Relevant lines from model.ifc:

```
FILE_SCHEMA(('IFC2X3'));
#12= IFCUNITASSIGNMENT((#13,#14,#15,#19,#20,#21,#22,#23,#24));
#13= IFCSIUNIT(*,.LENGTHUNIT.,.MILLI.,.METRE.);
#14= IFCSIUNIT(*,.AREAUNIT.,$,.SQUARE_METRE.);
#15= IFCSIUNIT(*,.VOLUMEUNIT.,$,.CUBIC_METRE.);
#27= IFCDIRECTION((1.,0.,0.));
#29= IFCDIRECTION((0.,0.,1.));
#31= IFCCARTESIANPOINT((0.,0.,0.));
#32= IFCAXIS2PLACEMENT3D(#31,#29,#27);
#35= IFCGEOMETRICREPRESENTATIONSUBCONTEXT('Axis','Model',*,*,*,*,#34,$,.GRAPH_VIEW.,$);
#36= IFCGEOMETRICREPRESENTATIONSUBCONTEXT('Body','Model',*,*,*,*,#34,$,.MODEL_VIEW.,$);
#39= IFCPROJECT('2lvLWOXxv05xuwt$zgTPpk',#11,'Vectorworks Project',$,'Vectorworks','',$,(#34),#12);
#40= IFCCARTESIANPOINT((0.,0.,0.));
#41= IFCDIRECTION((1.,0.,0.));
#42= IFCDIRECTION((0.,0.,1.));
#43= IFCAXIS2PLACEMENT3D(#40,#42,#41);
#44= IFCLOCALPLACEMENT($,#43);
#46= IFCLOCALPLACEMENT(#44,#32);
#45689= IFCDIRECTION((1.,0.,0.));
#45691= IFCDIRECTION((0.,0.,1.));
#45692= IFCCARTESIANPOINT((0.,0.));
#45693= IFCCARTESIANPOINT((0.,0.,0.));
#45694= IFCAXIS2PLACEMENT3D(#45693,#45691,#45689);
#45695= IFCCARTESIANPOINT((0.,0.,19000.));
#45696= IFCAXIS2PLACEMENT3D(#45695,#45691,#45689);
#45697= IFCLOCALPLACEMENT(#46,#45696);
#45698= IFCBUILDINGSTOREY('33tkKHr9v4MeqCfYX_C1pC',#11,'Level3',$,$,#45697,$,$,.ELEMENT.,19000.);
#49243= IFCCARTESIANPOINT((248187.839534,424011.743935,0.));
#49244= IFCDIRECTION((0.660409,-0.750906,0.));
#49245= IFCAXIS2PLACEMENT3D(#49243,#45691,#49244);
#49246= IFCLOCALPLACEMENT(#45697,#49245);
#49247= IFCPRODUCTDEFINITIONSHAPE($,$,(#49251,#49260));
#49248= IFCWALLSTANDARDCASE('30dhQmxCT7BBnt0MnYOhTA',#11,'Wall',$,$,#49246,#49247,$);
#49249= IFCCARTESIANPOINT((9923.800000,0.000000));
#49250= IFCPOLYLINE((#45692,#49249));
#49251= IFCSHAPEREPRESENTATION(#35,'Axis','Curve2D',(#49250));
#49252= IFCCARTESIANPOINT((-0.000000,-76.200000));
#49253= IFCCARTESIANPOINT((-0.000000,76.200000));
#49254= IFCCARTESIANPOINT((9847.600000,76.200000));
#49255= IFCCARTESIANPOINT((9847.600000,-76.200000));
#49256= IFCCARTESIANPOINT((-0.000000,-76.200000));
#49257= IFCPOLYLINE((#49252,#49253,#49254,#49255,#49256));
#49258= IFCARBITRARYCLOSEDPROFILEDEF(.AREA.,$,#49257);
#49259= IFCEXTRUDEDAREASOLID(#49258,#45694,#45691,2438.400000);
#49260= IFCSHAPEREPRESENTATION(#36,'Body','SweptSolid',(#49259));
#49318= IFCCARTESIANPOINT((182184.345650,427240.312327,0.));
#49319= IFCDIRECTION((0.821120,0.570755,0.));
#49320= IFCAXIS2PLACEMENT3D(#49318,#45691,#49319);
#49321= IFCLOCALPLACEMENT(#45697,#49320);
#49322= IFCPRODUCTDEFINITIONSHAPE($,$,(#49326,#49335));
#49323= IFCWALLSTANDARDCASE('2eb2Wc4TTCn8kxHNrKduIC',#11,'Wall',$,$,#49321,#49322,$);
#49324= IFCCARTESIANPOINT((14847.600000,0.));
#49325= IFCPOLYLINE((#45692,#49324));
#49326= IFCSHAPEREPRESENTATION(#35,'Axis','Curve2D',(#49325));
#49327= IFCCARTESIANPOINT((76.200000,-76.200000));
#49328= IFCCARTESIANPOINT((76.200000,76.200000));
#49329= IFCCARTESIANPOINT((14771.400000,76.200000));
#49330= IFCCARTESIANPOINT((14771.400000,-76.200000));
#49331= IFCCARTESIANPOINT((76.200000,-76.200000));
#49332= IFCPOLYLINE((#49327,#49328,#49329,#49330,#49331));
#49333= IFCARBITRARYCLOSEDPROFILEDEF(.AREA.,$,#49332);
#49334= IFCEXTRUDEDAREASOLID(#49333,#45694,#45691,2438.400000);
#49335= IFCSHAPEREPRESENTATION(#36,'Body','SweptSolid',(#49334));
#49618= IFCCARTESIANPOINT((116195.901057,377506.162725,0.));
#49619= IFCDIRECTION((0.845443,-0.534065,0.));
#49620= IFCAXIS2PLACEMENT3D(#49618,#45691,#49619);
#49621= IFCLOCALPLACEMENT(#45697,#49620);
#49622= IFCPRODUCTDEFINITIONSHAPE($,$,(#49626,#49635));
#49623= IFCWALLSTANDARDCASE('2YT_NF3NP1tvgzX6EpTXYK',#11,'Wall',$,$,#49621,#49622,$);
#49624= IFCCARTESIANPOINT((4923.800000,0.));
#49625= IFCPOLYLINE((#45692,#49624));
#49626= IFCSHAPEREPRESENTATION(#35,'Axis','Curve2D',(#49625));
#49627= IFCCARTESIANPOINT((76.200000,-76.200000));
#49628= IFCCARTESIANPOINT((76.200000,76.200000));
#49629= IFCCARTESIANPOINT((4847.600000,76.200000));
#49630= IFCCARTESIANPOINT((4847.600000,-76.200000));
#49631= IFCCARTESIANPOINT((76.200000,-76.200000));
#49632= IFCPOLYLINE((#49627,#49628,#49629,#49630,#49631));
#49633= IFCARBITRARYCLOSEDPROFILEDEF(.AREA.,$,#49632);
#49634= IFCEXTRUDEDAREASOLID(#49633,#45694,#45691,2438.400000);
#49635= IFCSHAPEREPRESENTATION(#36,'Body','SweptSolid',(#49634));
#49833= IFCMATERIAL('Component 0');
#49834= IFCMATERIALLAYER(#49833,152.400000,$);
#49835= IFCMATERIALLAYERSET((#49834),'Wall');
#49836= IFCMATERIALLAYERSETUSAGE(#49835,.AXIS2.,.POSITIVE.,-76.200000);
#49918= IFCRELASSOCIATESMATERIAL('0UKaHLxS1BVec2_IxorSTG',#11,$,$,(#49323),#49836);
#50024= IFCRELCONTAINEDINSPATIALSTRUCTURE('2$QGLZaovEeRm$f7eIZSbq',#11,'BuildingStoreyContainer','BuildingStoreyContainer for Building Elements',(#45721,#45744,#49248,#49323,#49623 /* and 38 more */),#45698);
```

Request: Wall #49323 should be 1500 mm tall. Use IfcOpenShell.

```python
import ifcopenshell
import ifcopenshell.geom
import ifcopenshell.util.representation
import ifcopenshell.util.shape
import ifcopenshell.util.unit

model = ifcopenshell.open("model.ifc")
unit_scale = ifcopenshell.util.unit.calculate_unit_scale(model)
settings = ifcopenshell.geom.settings()


def volume(element):
    """Net volume in cubic metres, openings subtracted."""
    shape = ifcopenshell.geom.create_shape(settings, element)
    return ifcopenshell.util.shape.get_volume(shape.geometry)


wall = model.by_guid("2eb2Wc4TTCn8kxHNrKduIC")
before = volume(wall)

body = ifcopenshell.util.representation.get_representation(wall, "Model", "Body")
solid = body.Items[0]
old_height = solid.Depth
solid.Depth = 1.5 / unit_scale
after = volume(wall)

print(f"height {old_height:g} -> {solid.Depth:g}, volume {before:.3f} -> {after:.3f} m3")

model.write("model_updated.ifc")
```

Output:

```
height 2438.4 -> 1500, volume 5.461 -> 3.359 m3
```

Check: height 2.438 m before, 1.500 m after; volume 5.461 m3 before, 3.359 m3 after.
